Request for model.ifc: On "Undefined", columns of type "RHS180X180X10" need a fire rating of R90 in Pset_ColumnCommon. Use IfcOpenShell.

First a look at what the model holds.

```python
import ifcopenshell
import ifcopenshell.util.element

model = ifcopenshell.open("model.ifc")
print(model.schema)
storey = next(s for s in model.by_type("IfcBuildingStorey") if s.Name == "Undefined")
columns = [e for e in ifcopenshell.util.element.get_decomposition(storey) if e.is_a("IfcColumn")]
seen = {}
for e in columns:
    element_type = ifcopenshell.util.element.get_type(e)
    key = (element_type.Name if element_type != e and element_type else None, ifcopenshell.util.element.get_pset(e, "Pset_ColumnCommon", "FireRating"))
    seen[key] = seen.get(key, 0) + 1
for (name, value), count in sorted(seen.items(), key=str):
    print(count, "x", name, "|", value)
```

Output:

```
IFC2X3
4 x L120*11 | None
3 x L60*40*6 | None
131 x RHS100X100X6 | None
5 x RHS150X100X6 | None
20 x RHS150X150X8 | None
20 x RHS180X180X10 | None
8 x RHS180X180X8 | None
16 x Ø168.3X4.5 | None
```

```python
import ifcopenshell
import ifcopenshell.api.pset
import ifcopenshell.util.element

model = ifcopenshell.open("model.ifc")

storey = next(s for s in model.by_type("IfcBuildingStorey") if s.Name == "Undefined")
columns = [e for e in ifcopenshell.util.element.get_decomposition(storey) if e.is_a("IfcColumn")]

count = 0
for e in columns:
    element_type = ifcopenshell.util.element.get_type(e)
    if element_type in (None, e) or element_type.Name != "RHS180X180X10":
        continue
    found = ifcopenshell.util.element.get_pset(e, "Pset_ColumnCommon", should_inherit=False)
    if found:
        pset = model.by_id(found["id"])
        if len(ifcopenshell.util.element.get_elements_by_pset(pset)) > 1:
            pset = ifcopenshell.api.pset.unshare_pset(model, products=[e], pset=pset)[0]
    else:
        pset = ifcopenshell.api.pset.add_pset(model, product=e, name="Pset_ColumnCommon")
    ifcopenshell.api.pset.edit_pset(model, pset=pset, properties={"FireRating": "R90"})
    count += 1

print(count, "columns updated")

model.write("model-out.ifc")
```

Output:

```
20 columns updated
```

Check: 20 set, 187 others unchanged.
